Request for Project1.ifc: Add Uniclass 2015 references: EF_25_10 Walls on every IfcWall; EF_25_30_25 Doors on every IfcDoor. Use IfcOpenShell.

First a look at what the model holds.

```python
import ifcopenshell

model = ifcopenshell.open("Project1.ifc")
print(model.schema)
print("classifications:", [c.Name for c in model.by_type("IfcClassification")])
for ifc_class in ("IfcDoor", "IfcRoof", "IfcStair", "IfcWall", "IfcWindow"):
    print(ifc_class, len(model.by_type(ifc_class)))
```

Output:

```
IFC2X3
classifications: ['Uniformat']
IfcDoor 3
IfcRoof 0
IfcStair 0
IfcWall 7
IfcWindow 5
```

```python
import ifcopenshell
import ifcopenshell.api.classification

model = ifcopenshell.open("Project1.ifc")

# IFC2X3 requires Source and Edition and has no link from the project to the system.
system = model.create_entity("IfcClassification", Source="NBS", Edition="2015", Name="Uniclass 2015")

codes = {
    "IfcWall": ("EF_25_10", "Walls"),
    "IfcDoor": ("EF_25_30_25", "Doors"),
}
for ifc_class, (code, name) in codes.items():
    products = model.by_type(ifc_class)
    ifcopenshell.api.classification.add_reference(
        model, products=products, classification=system, identification=code, name=name
    )
    print(code, len(products))

model.write("Project1_edited.ifc")
```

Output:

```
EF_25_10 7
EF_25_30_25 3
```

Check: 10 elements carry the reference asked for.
